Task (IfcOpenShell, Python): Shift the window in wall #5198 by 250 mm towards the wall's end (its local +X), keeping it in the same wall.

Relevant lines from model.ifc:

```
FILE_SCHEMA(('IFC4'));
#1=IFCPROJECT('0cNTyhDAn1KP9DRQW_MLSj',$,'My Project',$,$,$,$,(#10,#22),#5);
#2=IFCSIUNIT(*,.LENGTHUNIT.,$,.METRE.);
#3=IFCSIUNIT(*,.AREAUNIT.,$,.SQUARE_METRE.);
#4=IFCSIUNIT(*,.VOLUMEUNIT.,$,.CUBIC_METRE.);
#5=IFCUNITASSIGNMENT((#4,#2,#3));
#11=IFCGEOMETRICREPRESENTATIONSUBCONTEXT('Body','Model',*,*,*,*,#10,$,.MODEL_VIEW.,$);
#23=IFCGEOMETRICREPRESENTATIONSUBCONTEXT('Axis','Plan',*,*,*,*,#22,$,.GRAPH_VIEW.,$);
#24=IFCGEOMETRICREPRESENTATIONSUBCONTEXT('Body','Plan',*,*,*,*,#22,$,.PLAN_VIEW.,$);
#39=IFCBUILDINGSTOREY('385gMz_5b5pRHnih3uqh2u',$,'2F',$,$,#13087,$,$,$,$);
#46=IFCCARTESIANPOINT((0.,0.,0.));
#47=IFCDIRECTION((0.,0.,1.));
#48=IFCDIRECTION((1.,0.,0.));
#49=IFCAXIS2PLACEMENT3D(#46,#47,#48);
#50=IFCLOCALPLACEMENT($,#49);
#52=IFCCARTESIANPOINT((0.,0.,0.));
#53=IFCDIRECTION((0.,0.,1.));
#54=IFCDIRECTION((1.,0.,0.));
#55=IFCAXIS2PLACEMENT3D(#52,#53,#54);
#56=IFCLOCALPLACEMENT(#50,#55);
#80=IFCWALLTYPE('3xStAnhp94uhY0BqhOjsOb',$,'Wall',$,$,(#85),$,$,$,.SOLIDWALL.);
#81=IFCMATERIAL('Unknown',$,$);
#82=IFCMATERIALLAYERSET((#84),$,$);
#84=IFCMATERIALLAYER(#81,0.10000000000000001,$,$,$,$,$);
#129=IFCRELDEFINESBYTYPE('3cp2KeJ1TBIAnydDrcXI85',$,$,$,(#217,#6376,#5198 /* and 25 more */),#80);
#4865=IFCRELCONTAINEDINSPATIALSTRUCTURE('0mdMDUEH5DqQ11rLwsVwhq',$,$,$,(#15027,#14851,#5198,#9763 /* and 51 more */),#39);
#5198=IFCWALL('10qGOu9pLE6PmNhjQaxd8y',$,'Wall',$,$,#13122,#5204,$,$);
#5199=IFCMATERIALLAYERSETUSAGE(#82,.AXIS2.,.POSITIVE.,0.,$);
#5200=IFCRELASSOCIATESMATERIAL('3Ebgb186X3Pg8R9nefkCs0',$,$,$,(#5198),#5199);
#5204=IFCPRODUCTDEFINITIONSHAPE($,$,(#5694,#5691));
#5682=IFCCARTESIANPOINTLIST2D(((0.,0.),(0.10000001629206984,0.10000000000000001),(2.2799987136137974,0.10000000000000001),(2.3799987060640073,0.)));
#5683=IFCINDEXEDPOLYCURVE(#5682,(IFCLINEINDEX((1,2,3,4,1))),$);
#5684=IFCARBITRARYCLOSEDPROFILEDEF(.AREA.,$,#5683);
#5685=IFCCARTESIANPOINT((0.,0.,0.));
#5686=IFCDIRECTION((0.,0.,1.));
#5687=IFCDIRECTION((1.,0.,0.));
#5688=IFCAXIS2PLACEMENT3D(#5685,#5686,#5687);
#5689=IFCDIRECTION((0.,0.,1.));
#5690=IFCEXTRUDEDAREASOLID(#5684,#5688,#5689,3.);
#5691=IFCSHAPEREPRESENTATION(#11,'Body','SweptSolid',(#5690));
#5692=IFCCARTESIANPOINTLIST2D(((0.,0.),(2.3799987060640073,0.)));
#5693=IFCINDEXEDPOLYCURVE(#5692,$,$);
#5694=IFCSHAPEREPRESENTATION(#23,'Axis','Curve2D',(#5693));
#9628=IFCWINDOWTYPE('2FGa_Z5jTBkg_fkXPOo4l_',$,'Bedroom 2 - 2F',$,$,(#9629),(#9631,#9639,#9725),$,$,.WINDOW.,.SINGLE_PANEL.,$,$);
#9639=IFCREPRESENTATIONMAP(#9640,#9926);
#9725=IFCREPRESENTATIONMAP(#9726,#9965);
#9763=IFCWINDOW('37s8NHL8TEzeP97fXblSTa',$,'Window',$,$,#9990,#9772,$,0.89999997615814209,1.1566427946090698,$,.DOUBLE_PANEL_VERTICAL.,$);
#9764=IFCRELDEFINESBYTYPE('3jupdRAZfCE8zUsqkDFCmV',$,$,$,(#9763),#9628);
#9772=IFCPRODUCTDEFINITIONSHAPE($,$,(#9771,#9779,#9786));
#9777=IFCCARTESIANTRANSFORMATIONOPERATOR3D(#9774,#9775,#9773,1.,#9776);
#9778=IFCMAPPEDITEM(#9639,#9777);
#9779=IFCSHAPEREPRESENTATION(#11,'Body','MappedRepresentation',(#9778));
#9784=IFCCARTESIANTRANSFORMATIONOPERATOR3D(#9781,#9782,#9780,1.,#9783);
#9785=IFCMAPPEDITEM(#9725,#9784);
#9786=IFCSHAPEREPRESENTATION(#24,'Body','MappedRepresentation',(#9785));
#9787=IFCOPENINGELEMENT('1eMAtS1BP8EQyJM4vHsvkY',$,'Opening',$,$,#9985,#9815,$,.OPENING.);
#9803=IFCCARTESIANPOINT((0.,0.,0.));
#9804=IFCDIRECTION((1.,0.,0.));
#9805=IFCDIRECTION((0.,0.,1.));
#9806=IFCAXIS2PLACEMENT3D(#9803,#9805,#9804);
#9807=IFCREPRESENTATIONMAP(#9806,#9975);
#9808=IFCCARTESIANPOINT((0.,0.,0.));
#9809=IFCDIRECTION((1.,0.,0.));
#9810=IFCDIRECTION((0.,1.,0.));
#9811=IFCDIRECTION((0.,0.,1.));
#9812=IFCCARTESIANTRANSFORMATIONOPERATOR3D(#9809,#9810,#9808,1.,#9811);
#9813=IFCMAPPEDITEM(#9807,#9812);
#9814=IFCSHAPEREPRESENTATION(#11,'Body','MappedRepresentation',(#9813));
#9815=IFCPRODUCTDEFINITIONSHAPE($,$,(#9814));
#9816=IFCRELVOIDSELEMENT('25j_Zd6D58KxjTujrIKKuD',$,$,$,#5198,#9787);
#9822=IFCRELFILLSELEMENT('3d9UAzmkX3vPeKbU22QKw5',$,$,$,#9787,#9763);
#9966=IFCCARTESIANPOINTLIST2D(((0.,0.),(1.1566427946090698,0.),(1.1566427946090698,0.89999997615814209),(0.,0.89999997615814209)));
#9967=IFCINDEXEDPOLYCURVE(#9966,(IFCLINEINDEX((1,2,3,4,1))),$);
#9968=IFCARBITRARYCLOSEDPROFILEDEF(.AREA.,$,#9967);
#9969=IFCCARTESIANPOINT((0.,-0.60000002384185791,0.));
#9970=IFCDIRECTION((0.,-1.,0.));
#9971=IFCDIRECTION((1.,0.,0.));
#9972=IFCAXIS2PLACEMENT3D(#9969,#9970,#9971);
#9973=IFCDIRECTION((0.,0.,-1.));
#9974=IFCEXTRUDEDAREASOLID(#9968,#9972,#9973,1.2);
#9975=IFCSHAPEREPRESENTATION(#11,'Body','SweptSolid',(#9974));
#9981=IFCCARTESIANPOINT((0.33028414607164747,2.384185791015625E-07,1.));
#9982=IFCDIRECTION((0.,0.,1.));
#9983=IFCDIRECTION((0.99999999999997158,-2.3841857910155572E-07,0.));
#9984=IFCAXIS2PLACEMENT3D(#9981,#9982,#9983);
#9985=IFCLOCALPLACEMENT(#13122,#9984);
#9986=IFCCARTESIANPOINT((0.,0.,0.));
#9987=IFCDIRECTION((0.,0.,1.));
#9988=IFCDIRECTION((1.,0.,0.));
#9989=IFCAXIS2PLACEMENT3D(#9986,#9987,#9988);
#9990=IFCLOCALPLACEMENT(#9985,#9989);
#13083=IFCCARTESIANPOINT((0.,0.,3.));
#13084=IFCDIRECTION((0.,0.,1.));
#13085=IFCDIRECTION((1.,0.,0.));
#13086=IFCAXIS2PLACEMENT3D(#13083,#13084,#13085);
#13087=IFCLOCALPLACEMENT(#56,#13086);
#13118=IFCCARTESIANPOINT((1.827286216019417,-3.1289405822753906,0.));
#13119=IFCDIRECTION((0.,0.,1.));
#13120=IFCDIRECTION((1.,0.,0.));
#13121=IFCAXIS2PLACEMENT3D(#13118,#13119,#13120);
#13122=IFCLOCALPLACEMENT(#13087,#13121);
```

```python
import ifcopenshell
import ifcopenshell.api.geometry
import ifcopenshell.util.placement
import ifcopenshell.util.unit

model = ifcopenshell.open("model.ifc")
unit_scale = ifcopenshell.util.unit.calculate_unit_scale(model)

window = model.by_id(9763)
opening = window.FillsVoids[0].RelatingOpeningElement
wall = opening.VoidsElements[0].RelatingBuildingElement

wall_matrix = ifcopenshell.util.placement.get_local_placement(wall.ObjectPlacement)
shift = wall_matrix[:3, 0] * 0.25 / unit_scale
before = ifcopenshell.util.placement.get_local_placement(window.ObjectPlacement)[:3, 3].copy()

# The window is placed relative to its opening, so it follows when the opening moves.
matrix = ifcopenshell.util.placement.get_local_placement(opening.ObjectPlacement)
matrix[:3, 3] += shift
ifcopenshell.api.geometry.edit_object_placement(
    model, product=opening, matrix=matrix, is_si=False, should_transform_children=True
)

after = ifcopenshell.util.placement.get_local_placement(window.ObjectPlacement)[:3, 3]
print("window moved by", (after - before).round(3) + 0.0)

model.write("model_updated.ifc")
```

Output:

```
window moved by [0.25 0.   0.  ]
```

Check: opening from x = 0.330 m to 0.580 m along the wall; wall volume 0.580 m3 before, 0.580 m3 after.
